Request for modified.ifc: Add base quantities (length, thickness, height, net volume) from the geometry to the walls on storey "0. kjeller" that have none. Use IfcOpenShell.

First a look at what the model holds.

```python
import ifcopenshell
import ifcopenshell.util.element
import ifcopenshell.util.unit

model = ifcopenshell.open("modified.ifc")
print(model.schema)
for unit_type in ("LENGTHUNIT", "AREAUNIT", "VOLUMEUNIT"):
    print(unit_type, ifcopenshell.util.unit.calculate_unit_scale(model, unit_type))
storey = next(s for s in model.by_type("IfcBuildingStorey") if s.Name == "0. kjeller")
walls = [e for e in ifcopenshell.util.element.get_decomposition(storey) if e.is_a("IfcWall")]
for e in sorted(walls, key=lambda e: e.id()):
    print(e.id(), e.is_a(), e.Name, list(ifcopenshell.util.element.get_psets(e, qtos_only=True)), sep=" | ")
```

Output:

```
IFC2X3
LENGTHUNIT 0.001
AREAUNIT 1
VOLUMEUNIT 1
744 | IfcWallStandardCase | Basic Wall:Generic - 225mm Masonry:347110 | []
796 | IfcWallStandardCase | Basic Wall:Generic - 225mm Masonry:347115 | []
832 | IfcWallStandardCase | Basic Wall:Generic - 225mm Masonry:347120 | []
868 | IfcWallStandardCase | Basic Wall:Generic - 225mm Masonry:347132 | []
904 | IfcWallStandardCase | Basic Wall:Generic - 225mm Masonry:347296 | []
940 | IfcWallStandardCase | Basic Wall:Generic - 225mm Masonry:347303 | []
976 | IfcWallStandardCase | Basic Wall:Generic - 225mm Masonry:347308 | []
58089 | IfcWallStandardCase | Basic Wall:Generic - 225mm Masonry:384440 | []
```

```python
import ifcopenshell
import ifcopenshell.api.pset
import ifcopenshell.geom
import ifcopenshell.util.element
import ifcopenshell.util.shape
import ifcopenshell.util.unit

model = ifcopenshell.open("modified.ifc")
unit_scale = ifcopenshell.util.unit.calculate_unit_scale(model)
volume_scale = ifcopenshell.util.unit.calculate_unit_scale(model, "VOLUMEUNIT")
settings = ifcopenshell.geom.settings()

storey = next(s for s in model.by_type("IfcBuildingStorey") if s.Name == "0. kjeller")
walls = [e for e in ifcopenshell.util.element.get_decomposition(storey) if e.is_a("IfcWall")]

for e in sorted(walls, key=lambda e: e.id()):
    if ifcopenshell.util.element.get_psets(e, qtos_only=True, should_inherit=False):
        continue
    # Geometry comes back in metres, in the element's own axes.
    shape = ifcopenshell.geom.create_shape(settings, e)
    values = {
        "Length": ifcopenshell.util.shape.get_x(shape.geometry) / unit_scale,
        "Width": ifcopenshell.util.shape.get_y(shape.geometry) / unit_scale,
        "Height": ifcopenshell.util.shape.get_z(shape.geometry) / unit_scale,
        "NetVolume": ifcopenshell.util.shape.get_volume(shape.geometry) / volume_scale,
    }
    qto = ifcopenshell.api.pset.add_qto(model, product=e, name="BaseQuantities")
    ifcopenshell.api.pset.edit_qto(model, qto=qto, properties=values)
    print(e.id(), {k: round(v, 3) for k, v in values.items()})

model.write("modified_v2.ifc")
```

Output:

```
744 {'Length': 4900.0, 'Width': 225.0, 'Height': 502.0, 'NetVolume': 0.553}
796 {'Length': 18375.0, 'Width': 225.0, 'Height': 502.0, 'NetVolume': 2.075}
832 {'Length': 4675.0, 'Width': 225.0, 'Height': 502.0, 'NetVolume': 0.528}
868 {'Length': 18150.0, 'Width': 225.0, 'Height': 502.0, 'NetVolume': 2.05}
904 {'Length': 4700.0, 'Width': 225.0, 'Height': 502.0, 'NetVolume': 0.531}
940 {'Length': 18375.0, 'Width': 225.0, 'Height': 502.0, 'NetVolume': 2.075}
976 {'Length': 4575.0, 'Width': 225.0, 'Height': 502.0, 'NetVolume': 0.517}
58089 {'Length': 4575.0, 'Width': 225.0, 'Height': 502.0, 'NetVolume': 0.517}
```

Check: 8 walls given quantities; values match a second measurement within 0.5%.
